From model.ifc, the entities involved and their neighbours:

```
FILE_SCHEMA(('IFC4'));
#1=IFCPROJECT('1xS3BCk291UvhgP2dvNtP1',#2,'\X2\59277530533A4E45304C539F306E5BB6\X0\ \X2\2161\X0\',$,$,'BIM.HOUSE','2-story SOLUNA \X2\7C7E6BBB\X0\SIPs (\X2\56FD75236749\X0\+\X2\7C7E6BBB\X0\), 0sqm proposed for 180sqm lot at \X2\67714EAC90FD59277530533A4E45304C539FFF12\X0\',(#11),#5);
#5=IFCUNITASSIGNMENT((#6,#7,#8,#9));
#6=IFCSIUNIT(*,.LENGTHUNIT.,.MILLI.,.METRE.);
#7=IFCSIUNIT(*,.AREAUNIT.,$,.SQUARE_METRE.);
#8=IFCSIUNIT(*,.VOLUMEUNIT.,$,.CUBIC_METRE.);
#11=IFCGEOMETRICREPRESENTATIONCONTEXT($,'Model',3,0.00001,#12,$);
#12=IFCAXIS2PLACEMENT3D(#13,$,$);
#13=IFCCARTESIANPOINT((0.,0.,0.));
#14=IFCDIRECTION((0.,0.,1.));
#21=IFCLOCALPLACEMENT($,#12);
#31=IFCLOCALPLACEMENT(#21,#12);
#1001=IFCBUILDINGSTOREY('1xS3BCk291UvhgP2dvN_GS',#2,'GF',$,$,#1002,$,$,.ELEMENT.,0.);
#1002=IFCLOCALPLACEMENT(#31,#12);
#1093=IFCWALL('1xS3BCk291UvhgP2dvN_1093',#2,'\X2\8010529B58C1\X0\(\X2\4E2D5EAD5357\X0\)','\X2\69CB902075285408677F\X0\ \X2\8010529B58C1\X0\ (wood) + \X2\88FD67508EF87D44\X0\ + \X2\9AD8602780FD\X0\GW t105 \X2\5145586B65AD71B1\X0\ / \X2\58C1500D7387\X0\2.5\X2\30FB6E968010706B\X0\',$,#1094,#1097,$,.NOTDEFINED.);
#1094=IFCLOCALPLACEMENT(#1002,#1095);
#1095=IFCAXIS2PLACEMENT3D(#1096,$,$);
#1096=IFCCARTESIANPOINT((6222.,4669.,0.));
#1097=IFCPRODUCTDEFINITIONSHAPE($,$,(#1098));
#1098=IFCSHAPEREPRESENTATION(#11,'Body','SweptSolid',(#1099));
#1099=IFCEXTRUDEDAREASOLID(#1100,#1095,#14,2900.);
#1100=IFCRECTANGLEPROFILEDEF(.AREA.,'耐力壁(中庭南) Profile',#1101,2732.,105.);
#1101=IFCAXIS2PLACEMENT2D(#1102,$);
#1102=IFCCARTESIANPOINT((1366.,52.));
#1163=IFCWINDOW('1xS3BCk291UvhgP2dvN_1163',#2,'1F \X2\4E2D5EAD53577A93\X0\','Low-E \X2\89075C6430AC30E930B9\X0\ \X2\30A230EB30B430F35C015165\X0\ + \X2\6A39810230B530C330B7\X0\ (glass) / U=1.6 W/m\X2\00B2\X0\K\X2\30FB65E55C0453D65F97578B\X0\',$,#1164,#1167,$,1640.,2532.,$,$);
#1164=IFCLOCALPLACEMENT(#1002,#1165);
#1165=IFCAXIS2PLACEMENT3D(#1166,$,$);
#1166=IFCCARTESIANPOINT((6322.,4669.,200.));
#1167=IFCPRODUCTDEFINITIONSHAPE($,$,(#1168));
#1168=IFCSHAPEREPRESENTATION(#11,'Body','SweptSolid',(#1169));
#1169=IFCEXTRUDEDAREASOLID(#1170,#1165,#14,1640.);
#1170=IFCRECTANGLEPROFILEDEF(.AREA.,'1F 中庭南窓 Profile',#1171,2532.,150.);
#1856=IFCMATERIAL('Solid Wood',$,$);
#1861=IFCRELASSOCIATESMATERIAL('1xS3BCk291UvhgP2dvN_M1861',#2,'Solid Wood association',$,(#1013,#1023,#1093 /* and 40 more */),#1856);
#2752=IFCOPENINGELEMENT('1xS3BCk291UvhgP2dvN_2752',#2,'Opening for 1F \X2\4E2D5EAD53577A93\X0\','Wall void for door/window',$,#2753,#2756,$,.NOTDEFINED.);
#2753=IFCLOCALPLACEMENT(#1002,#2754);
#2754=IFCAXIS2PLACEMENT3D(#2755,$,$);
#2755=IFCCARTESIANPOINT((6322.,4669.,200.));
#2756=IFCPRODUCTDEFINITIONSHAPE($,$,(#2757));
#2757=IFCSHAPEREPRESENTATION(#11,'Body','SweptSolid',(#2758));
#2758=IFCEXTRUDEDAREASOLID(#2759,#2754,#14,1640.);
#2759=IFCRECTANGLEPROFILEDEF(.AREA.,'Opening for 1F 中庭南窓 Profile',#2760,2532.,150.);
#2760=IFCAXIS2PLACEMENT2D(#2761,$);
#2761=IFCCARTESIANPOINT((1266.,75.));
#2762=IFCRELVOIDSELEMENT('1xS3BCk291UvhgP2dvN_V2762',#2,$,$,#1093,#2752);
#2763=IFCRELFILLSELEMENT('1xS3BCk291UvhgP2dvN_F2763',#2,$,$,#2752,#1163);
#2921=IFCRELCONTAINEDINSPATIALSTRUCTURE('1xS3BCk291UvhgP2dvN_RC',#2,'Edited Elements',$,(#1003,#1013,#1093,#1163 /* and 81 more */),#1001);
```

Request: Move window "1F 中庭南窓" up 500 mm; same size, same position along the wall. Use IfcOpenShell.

```python
import numpy as np
import ifcopenshell
import ifcopenshell.api.geometry
import ifcopenshell.util.placement
import ifcopenshell.util.unit

model = ifcopenshell.open("model.ifc")
unit_scale = ifcopenshell.util.unit.calculate_unit_scale(model)

window = model.by_guid("1xS3BCk291UvhgP2dvN_1163")
opening = window.FillsVoids[0].RelatingOpeningElement
dz = 500.0

shift = np.array([0.0, 0.0, dz])
# The window is not placed relative to its opening, so move both.
for product in (opening, window):
    matrix = ifcopenshell.util.placement.get_local_placement(product.ObjectPlacement)
    matrix[:3, 3] += shift
    ifcopenshell.api.geometry.edit_object_placement(model, product=product, matrix=matrix, is_si=False)

print(f"moved by {dz * unit_scale:+.3f} m")

model.write("model-out.ifc")
```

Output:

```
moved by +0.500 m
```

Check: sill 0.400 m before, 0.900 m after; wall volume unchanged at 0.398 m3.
